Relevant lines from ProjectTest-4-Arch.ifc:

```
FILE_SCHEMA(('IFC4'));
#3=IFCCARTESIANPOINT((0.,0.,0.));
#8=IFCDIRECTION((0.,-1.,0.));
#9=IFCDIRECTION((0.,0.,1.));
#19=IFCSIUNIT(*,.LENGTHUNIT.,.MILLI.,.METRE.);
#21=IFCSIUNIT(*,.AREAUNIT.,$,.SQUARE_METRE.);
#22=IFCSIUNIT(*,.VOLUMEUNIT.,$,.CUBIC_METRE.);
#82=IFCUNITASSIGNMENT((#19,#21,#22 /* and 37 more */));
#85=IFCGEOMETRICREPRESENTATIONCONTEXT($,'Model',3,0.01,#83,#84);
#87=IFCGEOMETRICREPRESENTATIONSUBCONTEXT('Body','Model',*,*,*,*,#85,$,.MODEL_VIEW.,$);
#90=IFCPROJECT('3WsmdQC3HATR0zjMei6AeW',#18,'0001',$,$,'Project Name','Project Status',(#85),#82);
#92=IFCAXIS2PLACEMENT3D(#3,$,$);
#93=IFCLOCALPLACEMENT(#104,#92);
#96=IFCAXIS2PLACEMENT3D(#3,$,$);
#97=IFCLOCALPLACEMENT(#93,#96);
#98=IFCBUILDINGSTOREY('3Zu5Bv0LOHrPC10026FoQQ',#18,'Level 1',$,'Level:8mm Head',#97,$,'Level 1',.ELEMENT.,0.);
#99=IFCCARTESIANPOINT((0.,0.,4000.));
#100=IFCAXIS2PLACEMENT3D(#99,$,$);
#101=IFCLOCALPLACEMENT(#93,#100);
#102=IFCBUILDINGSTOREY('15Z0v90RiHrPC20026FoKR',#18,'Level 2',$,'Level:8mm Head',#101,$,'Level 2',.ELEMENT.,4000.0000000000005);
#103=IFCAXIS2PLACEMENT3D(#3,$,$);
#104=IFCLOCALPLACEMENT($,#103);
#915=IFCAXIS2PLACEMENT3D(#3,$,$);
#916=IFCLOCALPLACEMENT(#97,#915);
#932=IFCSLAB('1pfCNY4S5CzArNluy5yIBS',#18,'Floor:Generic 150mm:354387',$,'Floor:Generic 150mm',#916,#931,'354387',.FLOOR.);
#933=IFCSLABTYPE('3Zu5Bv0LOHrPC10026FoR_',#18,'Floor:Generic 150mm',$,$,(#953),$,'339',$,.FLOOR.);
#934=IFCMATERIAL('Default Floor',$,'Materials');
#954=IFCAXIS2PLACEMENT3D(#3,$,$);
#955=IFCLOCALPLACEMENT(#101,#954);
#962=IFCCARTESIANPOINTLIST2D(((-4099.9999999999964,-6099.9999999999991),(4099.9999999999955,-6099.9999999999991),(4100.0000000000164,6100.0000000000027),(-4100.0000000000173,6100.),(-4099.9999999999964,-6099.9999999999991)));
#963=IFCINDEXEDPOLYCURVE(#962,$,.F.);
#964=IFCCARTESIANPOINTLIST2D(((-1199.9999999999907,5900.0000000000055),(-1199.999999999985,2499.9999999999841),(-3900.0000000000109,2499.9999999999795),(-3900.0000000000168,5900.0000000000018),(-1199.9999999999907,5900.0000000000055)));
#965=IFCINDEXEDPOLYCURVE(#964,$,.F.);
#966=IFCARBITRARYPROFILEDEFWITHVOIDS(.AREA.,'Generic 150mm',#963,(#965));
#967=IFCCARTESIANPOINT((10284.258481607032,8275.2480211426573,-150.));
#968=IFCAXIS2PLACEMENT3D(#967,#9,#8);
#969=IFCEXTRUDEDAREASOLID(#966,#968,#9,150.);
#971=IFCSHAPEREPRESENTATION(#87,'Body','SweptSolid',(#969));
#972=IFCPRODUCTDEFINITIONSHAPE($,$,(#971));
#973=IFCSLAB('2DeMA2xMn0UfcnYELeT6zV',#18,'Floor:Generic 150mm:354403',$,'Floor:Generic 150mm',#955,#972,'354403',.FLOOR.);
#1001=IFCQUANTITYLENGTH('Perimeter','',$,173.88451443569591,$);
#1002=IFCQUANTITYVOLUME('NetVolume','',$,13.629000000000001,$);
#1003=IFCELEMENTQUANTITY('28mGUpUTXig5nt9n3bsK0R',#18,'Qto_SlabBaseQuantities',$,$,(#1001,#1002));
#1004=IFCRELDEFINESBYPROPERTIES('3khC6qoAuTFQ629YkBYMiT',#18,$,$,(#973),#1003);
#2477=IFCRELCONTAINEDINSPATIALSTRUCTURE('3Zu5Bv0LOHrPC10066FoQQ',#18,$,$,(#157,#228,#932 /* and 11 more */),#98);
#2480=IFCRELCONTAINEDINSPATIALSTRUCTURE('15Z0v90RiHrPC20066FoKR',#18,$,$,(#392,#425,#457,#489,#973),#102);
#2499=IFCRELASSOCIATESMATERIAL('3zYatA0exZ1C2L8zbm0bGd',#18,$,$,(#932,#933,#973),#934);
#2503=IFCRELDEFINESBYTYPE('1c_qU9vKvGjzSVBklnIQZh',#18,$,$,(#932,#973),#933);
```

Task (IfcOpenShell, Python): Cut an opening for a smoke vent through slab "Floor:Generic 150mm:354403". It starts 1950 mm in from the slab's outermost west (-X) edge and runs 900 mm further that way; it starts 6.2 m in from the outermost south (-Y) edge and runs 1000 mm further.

```python
import numpy as np
import ifcopenshell
import ifcopenshell.api.feature
import ifcopenshell.api.geometry
import ifcopenshell.api.pset
import ifcopenshell.api.root
import ifcopenshell.geom
import ifcopenshell.util.element
import ifcopenshell.util.placement
import ifcopenshell.util.representation
import ifcopenshell.util.shape
import ifcopenshell.util.unit

model = ifcopenshell.open("ProjectTest-4-Arch.ifc")
unit_scale = ifcopenshell.util.unit.calculate_unit_scale(model)
volume_scale = ifcopenshell.util.unit.calculate_unit_scale(model, "VOLUMEUNIT")
settings = ifcopenshell.geom.settings()


def volume(element):
    """Net volume in cubic metres, openings subtracted."""
    shape = ifcopenshell.geom.create_shape(settings, element)
    return ifcopenshell.util.shape.get_volume(shape.geometry)


slab = model.by_guid("2DeMA2xMn0UfcnYELeT6zV")
before = volume(slab)

# Extent in the slab's own axes, in metres. The edges named are its -X and -Y sides.
slab_shape = ifcopenshell.geom.create_shape(settings, slab)
vertices = ifcopenshell.util.shape.get_vertices(slab_shape.geometry)
x_min, y_min, bottom = vertices.min(axis=0)
top = vertices[:, 2].max()

opening = ifcopenshell.api.root.create_entity(model, ifc_class="IfcOpeningElement", name="Smoke vent opening", predefined_type="OPENING")
context = ifcopenshell.util.representation.get_context(model, "Model", "Body", "MODEL_VIEW")
width, depth = 0.9, 1
outline = [(0.0, 0.0), (width, 0.0), (width, depth), (0.0, depth), (0.0, 0.0)]
# Overshoot both faces by 50 mm so the cut is clean.
shape = ifcopenshell.api.geometry.add_slab_representation(
    model, context=context, depth=top - bottom + 0.1, polyline=outline
)
ifcopenshell.api.geometry.assign_representation(model, product=opening, representation=shape)

matrix = ifcopenshell.util.placement.get_local_placement(slab.ObjectPlacement)
matrix[:, 3] = matrix @ np.append(np.array([x_min + 1.95, y_min + 6.2, bottom - 0.05]) / unit_scale, 1.0)
ifcopenshell.api.geometry.edit_object_placement(model, product=opening, matrix=matrix, is_si=False)
ifcopenshell.api.feature.add_feature(model, feature=opening, element=slab)

after = volume(slab)

# Update the slab's stored quantities.
qto = model.by_id(ifcopenshell.util.element.get_pset(slab, "Qto_SlabBaseQuantities", should_inherit=False)["id"])
ifcopenshell.api.pset.edit_qto(model, qto=qto, properties={"NetVolume": after / volume_scale})

print(f"slab volume {before:.3f} -> {after:.3f} m3")

model.write("ProjectTest-4-Arch_edited.ifc")
```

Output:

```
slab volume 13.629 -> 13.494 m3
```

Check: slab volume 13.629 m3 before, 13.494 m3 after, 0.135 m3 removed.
